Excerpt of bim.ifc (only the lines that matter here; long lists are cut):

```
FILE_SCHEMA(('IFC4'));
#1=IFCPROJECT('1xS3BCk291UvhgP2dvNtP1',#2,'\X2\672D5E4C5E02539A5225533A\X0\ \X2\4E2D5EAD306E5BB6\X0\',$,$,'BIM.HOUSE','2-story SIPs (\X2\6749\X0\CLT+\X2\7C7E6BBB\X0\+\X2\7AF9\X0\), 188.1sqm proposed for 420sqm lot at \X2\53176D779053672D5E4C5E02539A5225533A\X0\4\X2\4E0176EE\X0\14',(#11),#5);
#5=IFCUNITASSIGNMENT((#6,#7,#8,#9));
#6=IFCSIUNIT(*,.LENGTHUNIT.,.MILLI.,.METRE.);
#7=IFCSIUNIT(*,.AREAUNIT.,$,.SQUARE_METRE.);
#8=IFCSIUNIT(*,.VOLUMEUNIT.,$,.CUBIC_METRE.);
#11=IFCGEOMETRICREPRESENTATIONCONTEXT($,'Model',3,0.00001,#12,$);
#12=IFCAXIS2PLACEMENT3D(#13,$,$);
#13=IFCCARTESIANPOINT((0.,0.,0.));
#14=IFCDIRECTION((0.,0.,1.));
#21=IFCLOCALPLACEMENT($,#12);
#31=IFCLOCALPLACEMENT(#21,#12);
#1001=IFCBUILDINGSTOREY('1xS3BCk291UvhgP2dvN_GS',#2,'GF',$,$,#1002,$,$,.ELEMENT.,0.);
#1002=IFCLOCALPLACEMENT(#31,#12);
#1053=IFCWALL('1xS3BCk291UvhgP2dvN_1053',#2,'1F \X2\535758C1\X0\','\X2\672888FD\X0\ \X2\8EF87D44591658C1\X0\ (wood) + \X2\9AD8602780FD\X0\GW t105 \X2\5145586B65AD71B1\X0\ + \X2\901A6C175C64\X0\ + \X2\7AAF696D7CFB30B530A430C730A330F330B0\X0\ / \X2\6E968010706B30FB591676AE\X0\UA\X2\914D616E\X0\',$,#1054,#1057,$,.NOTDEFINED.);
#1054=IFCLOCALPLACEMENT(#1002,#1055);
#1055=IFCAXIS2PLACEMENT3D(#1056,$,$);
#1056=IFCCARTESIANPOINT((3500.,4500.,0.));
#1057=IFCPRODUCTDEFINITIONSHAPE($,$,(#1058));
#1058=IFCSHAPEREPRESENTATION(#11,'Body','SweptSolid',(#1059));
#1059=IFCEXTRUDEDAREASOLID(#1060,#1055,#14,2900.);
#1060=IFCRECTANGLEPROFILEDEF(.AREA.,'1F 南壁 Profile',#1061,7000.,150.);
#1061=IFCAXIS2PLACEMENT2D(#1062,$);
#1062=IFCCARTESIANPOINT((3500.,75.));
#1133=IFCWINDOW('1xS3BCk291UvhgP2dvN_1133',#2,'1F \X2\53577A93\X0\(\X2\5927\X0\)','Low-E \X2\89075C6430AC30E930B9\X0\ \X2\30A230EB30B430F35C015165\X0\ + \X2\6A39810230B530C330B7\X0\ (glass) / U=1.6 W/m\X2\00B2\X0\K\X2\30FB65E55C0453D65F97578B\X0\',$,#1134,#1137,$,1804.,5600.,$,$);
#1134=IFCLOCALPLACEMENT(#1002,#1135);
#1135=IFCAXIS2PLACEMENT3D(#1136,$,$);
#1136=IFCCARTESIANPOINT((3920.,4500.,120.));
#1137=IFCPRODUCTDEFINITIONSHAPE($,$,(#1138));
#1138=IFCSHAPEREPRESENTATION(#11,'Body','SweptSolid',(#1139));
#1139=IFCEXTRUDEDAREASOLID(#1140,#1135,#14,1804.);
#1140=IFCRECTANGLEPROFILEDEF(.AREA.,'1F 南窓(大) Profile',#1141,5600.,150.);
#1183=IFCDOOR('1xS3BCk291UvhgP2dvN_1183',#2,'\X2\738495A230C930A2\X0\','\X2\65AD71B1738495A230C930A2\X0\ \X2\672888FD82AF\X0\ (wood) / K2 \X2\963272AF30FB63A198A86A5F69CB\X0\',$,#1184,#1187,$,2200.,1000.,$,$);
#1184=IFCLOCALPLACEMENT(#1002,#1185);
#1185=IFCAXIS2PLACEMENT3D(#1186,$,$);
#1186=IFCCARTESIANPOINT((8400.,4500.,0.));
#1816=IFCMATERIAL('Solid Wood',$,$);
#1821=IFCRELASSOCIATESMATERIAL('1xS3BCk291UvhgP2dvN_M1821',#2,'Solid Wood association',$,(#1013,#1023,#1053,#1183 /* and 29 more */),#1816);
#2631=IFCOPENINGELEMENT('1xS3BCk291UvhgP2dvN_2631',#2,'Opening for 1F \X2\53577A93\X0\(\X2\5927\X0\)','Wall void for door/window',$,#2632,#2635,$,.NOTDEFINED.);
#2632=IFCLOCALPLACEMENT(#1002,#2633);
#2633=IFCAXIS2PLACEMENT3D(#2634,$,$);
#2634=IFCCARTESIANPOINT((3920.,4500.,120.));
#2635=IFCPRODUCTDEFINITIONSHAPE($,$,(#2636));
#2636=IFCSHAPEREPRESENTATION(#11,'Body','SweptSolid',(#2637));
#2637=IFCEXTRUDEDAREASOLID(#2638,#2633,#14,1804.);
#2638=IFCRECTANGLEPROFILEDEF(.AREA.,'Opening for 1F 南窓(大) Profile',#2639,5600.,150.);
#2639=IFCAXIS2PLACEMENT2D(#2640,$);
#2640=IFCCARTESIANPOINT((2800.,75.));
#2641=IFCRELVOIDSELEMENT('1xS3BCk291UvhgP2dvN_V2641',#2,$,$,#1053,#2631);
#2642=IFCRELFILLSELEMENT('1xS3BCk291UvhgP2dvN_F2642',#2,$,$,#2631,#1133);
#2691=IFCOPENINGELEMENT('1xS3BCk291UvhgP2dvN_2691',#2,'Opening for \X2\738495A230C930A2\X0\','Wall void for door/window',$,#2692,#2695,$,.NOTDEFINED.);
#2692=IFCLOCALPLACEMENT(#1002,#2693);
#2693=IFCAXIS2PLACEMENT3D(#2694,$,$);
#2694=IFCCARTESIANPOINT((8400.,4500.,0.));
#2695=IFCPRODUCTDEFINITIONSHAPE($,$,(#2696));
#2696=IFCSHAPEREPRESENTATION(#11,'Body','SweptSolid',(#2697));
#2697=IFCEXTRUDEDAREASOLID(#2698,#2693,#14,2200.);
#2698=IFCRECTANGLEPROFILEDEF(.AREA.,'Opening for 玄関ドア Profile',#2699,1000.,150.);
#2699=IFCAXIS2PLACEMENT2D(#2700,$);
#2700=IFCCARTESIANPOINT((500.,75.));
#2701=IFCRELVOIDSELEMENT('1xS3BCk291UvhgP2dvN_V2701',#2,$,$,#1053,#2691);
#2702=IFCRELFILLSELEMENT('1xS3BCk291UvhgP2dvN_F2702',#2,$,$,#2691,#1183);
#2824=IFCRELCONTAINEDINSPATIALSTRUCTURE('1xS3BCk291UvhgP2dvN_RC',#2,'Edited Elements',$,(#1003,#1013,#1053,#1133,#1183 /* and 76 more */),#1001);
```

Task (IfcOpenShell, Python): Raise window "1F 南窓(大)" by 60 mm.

```python
import numpy as np
import ifcopenshell
import ifcopenshell.api.geometry
import ifcopenshell.util.placement
import ifcopenshell.util.unit

model = ifcopenshell.open("bim.ifc")
unit_scale = ifcopenshell.util.unit.calculate_unit_scale(model)

window = model.by_id(1133)
opening = window.FillsVoids[0].RelatingOpeningElement
dz = 60.0

shift = np.array([0.0, 0.0, dz])
# The window is not placed relative to its opening, so move both.
for product in (opening, window):
    matrix = ifcopenshell.util.placement.get_local_placement(product.ObjectPlacement)
    matrix[:3, 3] += shift
    ifcopenshell.api.geometry.edit_object_placement(model, product=product, matrix=matrix, is_si=False)

print(f"moved by {dz * unit_scale:+.3f} m")

model.write("bim_edited.ifc")
```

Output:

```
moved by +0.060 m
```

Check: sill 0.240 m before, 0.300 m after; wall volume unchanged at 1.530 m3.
